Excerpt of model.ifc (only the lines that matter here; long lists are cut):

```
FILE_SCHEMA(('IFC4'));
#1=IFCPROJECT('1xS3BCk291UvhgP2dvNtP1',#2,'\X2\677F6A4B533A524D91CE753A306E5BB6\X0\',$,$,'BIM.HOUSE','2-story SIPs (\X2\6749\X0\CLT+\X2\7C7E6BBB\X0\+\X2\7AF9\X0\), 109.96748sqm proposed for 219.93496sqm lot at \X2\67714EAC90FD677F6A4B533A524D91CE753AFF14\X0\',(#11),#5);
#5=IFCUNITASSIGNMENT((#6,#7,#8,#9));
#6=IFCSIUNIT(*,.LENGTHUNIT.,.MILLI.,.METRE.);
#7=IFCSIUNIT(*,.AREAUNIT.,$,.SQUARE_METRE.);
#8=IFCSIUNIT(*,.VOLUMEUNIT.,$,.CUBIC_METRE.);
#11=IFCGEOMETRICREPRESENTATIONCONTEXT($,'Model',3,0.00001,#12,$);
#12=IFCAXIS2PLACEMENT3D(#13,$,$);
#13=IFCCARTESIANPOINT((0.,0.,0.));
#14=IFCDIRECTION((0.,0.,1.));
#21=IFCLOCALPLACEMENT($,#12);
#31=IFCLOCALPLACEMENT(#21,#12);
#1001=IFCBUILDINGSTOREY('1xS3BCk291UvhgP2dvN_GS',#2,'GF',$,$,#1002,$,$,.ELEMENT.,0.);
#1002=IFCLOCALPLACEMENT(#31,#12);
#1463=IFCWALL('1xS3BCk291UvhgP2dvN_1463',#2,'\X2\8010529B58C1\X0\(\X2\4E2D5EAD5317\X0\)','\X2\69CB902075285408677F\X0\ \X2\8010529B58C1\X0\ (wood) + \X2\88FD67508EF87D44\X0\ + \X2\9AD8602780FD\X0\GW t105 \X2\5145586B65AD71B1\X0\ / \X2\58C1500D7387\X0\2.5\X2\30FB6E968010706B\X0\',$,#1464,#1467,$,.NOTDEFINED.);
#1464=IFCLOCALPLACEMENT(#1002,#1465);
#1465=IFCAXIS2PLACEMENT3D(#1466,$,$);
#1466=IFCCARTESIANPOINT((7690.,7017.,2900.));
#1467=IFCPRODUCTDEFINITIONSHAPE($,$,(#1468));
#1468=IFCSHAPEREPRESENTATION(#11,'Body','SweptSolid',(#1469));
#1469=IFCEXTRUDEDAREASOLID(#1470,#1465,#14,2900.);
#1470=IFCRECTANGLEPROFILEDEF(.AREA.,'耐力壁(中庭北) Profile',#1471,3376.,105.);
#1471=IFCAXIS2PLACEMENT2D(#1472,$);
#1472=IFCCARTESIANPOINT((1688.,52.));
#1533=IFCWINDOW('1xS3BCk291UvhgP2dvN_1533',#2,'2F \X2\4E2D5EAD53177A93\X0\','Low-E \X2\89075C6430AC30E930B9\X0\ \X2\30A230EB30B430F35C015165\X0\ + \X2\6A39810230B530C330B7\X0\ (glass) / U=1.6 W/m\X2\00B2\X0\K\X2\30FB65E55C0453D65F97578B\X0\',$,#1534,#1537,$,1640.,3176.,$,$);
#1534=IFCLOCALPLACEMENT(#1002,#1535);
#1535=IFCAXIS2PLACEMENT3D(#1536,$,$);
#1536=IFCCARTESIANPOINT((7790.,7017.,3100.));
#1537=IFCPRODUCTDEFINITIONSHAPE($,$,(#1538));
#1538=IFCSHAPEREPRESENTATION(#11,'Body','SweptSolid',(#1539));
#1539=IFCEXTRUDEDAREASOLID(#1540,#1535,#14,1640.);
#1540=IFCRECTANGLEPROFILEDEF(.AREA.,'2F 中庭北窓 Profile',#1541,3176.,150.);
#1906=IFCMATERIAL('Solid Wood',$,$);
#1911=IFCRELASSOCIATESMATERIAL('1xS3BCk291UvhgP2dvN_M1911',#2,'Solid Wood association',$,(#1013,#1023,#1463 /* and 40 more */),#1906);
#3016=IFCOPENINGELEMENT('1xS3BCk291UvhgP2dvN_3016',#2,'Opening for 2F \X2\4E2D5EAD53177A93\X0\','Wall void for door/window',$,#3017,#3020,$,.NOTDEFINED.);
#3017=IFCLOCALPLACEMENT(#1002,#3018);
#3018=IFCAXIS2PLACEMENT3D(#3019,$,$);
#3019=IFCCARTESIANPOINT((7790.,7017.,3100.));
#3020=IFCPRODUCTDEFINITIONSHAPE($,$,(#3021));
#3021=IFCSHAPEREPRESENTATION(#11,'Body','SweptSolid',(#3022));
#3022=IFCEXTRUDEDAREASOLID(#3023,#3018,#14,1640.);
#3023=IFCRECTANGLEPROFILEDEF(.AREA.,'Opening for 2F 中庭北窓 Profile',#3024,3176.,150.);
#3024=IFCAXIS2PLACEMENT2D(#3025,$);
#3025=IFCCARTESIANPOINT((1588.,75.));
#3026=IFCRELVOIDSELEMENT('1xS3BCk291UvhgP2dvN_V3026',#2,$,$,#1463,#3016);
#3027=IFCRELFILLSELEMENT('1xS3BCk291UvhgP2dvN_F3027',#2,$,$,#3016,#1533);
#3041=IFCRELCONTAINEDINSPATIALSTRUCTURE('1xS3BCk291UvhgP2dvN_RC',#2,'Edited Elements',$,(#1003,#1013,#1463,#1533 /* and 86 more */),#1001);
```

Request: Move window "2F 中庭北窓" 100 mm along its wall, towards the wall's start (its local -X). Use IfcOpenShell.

```python
import ifcopenshell
import ifcopenshell.api.geometry
import ifcopenshell.util.placement

model = ifcopenshell.open("model.ifc")

window = model.by_id(1533)
opening = window.FillsVoids[0].RelatingOpeningElement
wall = opening.VoidsElements[0].RelatingBuildingElement

wall_matrix = ifcopenshell.util.placement.get_local_placement(wall.ObjectPlacement)
shift = wall_matrix[:3, 0] * -100.0
before = ifcopenshell.util.placement.get_local_placement(window.ObjectPlacement)[:3, 3].copy()

# The window is not placed relative to its opening, so move both.
for product in (opening, window):
    matrix = ifcopenshell.util.placement.get_local_placement(product.ObjectPlacement)
    matrix[:3, 3] += shift
    ifcopenshell.api.geometry.edit_object_placement(model, product=product, matrix=matrix, is_si=False)

after = ifcopenshell.util.placement.get_local_placement(window.ObjectPlacement)[:3, 3]
print("window moved by", (after - before).round(3) + 0.0)

model.write("model_edited.ifc")
```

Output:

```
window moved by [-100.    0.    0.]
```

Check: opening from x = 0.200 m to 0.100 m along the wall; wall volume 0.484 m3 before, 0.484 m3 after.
